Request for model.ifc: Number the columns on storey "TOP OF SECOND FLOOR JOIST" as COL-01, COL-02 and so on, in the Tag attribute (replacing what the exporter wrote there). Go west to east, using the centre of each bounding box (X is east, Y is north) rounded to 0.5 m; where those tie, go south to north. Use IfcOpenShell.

First a look at what the model holds.

```python
import ifcopenshell
import ifcopenshell.util.element
import ifcopenshell.util.placement

model = ifcopenshell.open("model.ifc")
print(model.schema)
storey = next(s for s in model.by_type("IfcBuildingStorey") if s.Name == "TOP OF SECOND FLOOR JOIST")
columns = [e for e in ifcopenshell.util.element.get_decomposition(storey) if e.is_a("IfcColumn")]
for e in sorted(columns, key=lambda e: e.id()):
    origin = ifcopenshell.util.placement.get_local_placement(e.ObjectPlacement)[:3, 3]
    print(e.id(), e.Tag, e.Name, origin.round(2) + 0.0, sep=" | ")
```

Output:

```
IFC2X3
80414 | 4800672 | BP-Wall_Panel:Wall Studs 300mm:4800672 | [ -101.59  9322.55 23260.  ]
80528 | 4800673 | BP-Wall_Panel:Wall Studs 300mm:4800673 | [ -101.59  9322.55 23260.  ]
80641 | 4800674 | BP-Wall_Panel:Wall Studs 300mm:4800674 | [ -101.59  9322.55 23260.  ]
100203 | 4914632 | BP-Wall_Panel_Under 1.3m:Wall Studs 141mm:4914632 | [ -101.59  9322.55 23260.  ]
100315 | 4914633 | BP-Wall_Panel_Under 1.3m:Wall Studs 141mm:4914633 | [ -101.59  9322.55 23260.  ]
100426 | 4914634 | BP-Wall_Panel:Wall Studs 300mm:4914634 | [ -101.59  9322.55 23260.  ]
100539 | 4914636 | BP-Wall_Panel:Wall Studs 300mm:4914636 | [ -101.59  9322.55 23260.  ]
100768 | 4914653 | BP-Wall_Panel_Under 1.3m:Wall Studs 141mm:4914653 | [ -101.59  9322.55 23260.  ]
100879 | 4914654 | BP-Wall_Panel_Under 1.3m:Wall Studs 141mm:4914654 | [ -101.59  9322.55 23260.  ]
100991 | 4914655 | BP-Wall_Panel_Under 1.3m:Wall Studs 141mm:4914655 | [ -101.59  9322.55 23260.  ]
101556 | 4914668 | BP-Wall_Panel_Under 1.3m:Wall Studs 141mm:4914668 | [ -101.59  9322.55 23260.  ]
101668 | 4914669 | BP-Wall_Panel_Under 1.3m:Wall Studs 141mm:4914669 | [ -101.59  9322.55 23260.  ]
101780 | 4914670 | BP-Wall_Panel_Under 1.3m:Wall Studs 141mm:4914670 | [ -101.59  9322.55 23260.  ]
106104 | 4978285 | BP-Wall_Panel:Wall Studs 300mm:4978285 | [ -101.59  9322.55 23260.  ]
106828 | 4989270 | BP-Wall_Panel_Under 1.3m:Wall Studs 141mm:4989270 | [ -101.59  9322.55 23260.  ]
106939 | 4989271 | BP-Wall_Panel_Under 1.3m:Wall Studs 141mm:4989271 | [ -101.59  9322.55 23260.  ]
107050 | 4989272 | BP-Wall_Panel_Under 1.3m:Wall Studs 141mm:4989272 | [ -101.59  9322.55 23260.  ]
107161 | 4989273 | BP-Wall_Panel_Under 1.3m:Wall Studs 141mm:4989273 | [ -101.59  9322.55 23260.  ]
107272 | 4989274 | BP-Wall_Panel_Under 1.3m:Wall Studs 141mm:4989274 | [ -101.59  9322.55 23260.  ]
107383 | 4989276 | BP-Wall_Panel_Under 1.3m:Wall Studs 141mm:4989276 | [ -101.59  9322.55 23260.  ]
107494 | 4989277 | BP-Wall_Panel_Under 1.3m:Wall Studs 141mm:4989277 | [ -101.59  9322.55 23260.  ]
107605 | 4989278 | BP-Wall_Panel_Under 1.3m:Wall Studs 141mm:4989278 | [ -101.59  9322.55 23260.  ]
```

```python
import ifcopenshell
import ifcopenshell.geom
import ifcopenshell.util.element
import ifcopenshell.util.shape

model = ifcopenshell.open("model.ifc")
settings = ifcopenshell.geom.settings()
settings.set("use-world-coords", True)


def centre(element):
    shape = ifcopenshell.geom.create_shape(settings, element)
    return ifcopenshell.util.shape.get_bbox_centroid(shape.geometry)


storey = next(s for s in model.by_type("IfcBuildingStorey") if s.Name == "TOP OF SECOND FLOOR JOIST")
columns = [e for e in ifcopenshell.util.element.get_decomposition(storey) if e.is_a("IfcColumn")]

# Insertion points can sit at a corner or the storey origin, so sort by the geometry (in metres).
centres = {e: centre(e) for e in columns}
columns.sort(key=lambda e: (round(centres[e][0] / 0.5), centres[e][1]))

for i, e in enumerate(columns, start=1):
    number = f"COL-{i:02d}"
    e.Tag = number
    print(e.id(), number)

model.write("model_v2.ifc")
```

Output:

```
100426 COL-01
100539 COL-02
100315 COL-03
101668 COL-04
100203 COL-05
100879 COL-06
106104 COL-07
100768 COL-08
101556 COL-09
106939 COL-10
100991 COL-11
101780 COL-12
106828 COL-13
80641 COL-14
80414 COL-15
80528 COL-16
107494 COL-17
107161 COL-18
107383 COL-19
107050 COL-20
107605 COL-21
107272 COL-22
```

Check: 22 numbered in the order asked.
